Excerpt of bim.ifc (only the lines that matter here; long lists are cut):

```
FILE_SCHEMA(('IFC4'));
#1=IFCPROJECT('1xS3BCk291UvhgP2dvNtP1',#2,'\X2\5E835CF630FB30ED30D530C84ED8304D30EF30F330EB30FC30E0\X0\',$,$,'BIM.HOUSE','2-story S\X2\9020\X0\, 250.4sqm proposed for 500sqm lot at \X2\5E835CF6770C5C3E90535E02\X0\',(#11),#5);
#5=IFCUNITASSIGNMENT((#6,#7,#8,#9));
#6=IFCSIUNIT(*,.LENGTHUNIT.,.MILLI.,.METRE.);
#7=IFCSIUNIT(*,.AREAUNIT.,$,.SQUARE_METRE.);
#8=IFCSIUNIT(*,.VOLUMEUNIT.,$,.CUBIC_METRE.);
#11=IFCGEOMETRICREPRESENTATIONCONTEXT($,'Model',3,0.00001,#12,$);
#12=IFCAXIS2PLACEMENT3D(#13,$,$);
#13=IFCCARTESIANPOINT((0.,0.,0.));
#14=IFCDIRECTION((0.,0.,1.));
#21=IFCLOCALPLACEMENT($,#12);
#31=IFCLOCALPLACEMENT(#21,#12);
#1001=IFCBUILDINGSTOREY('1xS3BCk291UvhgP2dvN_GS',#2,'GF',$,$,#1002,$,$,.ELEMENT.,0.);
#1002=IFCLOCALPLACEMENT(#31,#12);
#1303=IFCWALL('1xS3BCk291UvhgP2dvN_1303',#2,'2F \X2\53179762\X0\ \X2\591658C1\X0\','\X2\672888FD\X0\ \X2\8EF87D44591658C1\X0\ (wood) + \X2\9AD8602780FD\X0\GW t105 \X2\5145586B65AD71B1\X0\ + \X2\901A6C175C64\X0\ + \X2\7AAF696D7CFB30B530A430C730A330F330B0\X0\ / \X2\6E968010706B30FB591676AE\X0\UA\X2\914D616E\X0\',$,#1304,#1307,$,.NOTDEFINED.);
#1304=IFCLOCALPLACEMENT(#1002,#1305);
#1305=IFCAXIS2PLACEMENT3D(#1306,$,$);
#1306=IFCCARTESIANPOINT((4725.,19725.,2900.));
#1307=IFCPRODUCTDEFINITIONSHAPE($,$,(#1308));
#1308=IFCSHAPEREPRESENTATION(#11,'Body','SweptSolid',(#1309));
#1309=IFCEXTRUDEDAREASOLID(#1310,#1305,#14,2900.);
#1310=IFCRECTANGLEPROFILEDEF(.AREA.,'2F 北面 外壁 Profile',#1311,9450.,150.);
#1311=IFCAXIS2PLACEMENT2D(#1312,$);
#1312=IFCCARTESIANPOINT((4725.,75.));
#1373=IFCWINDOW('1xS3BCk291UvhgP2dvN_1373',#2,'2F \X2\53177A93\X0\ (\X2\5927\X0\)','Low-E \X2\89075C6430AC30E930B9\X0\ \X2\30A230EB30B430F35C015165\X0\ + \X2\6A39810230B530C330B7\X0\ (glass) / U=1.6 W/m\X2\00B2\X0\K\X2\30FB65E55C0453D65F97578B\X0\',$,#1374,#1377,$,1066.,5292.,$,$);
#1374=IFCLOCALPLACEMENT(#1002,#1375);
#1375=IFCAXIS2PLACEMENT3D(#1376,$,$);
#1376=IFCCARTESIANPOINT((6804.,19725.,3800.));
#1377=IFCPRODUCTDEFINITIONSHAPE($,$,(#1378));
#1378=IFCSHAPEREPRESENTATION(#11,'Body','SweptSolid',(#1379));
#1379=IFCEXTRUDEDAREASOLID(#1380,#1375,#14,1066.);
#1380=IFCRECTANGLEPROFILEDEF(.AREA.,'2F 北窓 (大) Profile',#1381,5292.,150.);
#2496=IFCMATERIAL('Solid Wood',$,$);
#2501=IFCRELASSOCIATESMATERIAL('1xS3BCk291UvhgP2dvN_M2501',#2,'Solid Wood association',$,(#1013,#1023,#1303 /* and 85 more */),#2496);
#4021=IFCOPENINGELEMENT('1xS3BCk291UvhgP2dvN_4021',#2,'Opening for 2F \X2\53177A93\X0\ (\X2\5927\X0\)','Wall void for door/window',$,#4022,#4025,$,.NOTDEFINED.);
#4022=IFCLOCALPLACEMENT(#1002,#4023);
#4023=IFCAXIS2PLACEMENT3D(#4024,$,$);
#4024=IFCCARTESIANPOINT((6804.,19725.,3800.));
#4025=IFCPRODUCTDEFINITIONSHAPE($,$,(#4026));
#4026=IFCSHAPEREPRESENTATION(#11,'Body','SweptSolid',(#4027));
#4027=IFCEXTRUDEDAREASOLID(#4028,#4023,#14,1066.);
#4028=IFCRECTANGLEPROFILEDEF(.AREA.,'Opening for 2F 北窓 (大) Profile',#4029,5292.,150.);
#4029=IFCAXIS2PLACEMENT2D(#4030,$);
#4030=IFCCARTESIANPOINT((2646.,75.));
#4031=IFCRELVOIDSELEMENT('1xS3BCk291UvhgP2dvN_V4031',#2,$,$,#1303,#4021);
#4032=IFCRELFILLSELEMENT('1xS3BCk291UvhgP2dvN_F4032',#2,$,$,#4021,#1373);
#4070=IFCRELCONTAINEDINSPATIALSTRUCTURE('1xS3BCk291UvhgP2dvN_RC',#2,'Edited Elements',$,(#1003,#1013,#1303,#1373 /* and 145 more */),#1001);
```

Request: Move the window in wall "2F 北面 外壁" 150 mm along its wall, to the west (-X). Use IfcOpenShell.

```python
import ifcopenshell
import ifcopenshell.api.geometry
import ifcopenshell.util.placement
import ifcopenshell.util.unit

model = ifcopenshell.open("bim.ifc")
unit_scale = ifcopenshell.util.unit.calculate_unit_scale(model)

window = model.by_guid("1xS3BCk291UvhgP2dvN_1373")
opening = window.FillsVoids[0].RelatingOpeningElement
wall = opening.VoidsElements[0].RelatingBuildingElement

wall_matrix = ifcopenshell.util.placement.get_local_placement(wall.ObjectPlacement)
shift = wall_matrix[:3, 0] * -0.15 / unit_scale
before = ifcopenshell.util.placement.get_local_placement(window.ObjectPlacement)[:3, 3].copy()

# The window is not placed relative to its opening, so move both.
for product in (opening, window):
    matrix = ifcopenshell.util.placement.get_local_placement(product.ObjectPlacement)
    matrix[:3, 3] += shift
    ifcopenshell.api.geometry.edit_object_placement(model, product=product, matrix=matrix, is_si=False)

after = ifcopenshell.util.placement.get_local_placement(window.ObjectPlacement)[:3, 3]
print("window moved by", (after - before).round(3) + 0.0)

model.write("bim_rev.ifc")
```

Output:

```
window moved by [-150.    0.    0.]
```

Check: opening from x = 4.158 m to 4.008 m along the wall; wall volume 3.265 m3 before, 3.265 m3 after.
